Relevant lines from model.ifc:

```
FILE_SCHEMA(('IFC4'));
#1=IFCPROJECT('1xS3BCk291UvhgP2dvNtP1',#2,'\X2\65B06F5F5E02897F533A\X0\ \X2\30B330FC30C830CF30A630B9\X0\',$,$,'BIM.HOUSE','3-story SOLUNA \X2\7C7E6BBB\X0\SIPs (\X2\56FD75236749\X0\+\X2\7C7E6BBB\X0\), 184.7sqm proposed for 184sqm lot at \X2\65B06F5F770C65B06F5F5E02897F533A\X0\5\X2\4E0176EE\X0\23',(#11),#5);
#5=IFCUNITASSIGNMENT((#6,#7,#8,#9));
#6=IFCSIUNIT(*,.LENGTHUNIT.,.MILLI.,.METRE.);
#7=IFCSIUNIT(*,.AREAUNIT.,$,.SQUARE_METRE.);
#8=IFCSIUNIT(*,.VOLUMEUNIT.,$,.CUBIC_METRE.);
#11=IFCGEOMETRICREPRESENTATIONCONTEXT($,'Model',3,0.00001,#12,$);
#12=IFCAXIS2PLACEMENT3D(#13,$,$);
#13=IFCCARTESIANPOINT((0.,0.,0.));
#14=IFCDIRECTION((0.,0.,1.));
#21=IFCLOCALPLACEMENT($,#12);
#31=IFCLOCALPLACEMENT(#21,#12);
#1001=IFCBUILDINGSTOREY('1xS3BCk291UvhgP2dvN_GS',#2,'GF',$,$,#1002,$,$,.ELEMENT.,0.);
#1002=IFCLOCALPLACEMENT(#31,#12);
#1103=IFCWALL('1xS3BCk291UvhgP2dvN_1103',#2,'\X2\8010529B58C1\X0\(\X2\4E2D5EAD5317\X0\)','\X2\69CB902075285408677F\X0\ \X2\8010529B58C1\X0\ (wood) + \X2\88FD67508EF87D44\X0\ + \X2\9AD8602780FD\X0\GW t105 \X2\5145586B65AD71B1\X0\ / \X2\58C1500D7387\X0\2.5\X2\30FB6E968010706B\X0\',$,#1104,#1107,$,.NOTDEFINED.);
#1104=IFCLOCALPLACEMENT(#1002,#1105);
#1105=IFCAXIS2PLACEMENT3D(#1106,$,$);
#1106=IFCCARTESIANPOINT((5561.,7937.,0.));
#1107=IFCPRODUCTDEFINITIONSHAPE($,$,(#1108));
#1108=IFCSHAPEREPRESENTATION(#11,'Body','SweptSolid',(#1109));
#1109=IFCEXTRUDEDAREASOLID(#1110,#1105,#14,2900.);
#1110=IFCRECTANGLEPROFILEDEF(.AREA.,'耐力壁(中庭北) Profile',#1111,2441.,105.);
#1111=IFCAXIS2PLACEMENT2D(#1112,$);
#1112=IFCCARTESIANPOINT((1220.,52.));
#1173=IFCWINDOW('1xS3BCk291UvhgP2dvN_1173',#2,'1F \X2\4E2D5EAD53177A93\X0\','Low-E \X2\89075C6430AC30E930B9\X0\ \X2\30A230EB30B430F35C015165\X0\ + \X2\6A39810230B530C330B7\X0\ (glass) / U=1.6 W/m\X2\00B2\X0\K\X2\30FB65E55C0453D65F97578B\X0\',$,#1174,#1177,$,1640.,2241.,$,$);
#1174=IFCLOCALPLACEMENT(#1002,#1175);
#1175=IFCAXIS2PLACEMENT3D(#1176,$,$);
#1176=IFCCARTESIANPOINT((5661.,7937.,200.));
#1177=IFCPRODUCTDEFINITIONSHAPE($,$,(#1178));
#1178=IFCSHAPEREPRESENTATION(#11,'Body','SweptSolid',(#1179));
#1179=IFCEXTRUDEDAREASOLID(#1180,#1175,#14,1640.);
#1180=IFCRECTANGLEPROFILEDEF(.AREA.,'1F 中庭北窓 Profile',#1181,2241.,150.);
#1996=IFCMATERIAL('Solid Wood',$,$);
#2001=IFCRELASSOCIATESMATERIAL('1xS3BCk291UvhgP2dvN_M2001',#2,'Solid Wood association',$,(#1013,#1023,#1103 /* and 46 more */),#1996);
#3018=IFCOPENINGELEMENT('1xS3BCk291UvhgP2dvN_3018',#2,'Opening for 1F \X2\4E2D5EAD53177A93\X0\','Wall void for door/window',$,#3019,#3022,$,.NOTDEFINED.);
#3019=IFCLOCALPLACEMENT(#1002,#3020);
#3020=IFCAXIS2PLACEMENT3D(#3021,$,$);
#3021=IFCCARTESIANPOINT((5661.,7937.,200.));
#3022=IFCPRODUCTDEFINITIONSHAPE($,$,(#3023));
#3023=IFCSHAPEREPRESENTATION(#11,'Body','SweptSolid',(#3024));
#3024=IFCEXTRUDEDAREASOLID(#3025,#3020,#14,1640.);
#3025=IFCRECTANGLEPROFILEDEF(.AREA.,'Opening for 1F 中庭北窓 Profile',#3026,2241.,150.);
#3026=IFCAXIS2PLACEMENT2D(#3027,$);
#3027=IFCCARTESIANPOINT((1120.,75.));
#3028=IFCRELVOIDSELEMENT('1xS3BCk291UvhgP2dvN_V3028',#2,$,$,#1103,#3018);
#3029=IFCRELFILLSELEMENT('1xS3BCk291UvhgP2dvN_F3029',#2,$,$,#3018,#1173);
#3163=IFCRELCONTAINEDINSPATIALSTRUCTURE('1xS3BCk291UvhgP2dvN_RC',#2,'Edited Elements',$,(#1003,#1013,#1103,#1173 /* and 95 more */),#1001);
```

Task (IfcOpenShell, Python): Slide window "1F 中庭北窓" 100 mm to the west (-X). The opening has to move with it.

```python
import ifcopenshell
import ifcopenshell.api.geometry
import ifcopenshell.util.placement
import ifcopenshell.util.unit

model = ifcopenshell.open("model.ifc")
unit_scale = ifcopenshell.util.unit.calculate_unit_scale(model)

window = model.by_guid("1xS3BCk291UvhgP2dvN_1173")
opening = window.FillsVoids[0].RelatingOpeningElement
wall = opening.VoidsElements[0].RelatingBuildingElement

wall_matrix = ifcopenshell.util.placement.get_local_placement(wall.ObjectPlacement)
shift = wall_matrix[:3, 0] * -0.1 / unit_scale
before = ifcopenshell.util.placement.get_local_placement(window.ObjectPlacement)[:3, 3].copy()

# The window is not placed relative to its opening, so move both.
for product in (opening, window):
    matrix = ifcopenshell.util.placement.get_local_placement(product.ObjectPlacement)
    matrix[:3, 3] += shift
    ifcopenshell.api.geometry.edit_object_placement(model, product=product, matrix=matrix, is_si=False)

after = ifcopenshell.util.placement.get_local_placement(window.ObjectPlacement)[:3, 3]
print("window moved by", (after - before).round(3) + 0.0)

model.write("model_updated.ifc")
```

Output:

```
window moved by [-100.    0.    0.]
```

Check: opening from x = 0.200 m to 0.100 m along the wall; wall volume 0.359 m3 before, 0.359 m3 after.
